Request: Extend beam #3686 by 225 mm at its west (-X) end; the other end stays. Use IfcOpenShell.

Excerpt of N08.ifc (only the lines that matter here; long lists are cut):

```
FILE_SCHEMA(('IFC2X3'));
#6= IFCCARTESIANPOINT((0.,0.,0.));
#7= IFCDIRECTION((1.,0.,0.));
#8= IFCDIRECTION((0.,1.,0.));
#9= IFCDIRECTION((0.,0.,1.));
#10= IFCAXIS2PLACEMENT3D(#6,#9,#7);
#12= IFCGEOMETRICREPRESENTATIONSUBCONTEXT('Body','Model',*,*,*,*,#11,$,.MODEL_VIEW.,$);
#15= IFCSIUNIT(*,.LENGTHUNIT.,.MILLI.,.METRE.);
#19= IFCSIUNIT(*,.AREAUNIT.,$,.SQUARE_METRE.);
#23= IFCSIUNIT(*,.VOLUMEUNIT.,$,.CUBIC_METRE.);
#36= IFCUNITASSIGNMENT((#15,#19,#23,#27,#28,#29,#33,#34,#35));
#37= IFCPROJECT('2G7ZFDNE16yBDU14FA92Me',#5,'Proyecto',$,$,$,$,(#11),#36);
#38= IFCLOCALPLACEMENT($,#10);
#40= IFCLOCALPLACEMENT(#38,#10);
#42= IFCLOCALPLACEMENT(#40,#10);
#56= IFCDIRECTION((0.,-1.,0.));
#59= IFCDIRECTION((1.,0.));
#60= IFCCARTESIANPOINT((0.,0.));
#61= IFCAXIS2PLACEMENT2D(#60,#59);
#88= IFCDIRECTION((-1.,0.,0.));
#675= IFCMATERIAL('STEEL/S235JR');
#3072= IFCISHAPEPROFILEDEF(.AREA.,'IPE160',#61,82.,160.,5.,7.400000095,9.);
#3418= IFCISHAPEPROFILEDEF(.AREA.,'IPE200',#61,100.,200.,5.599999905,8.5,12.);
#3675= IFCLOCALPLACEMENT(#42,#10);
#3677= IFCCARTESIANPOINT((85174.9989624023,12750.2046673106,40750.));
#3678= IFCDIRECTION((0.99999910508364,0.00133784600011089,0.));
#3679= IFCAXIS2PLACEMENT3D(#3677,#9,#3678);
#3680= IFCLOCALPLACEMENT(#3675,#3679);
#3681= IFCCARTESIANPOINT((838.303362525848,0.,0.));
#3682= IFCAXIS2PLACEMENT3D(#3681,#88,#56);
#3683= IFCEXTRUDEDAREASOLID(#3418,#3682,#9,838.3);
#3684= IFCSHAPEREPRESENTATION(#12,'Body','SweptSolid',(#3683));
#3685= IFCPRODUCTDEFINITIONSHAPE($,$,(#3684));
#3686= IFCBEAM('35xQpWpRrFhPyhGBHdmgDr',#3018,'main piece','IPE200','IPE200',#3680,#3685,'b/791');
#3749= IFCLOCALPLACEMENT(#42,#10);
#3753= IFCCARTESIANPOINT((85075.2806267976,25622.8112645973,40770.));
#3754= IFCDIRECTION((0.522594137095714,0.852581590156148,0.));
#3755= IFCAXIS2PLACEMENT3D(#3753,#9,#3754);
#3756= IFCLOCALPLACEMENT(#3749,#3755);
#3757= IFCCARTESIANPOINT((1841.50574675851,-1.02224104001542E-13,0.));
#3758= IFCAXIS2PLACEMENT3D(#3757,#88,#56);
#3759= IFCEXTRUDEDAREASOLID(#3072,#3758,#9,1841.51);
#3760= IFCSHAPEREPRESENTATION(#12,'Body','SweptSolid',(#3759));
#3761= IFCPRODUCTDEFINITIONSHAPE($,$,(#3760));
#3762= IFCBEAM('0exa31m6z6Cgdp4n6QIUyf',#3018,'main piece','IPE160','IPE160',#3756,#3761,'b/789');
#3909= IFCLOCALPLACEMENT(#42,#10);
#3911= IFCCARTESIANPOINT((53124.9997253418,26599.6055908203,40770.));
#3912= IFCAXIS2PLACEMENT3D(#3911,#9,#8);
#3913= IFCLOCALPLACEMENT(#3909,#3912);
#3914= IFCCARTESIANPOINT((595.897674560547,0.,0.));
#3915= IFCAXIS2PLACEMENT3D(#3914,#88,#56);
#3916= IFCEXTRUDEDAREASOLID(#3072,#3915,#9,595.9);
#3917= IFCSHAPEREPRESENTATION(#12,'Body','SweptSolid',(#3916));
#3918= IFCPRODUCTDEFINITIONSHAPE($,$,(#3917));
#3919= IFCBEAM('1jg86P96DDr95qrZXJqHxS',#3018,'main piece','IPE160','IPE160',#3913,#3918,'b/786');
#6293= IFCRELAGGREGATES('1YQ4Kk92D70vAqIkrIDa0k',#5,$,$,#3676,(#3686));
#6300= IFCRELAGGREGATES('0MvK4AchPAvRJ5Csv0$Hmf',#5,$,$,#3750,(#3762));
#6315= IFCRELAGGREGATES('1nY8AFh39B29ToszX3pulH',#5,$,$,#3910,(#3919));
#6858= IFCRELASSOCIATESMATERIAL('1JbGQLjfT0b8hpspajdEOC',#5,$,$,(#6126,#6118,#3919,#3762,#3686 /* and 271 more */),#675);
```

```python
import ifcopenshell
import ifcopenshell.util.representation
import ifcopenshell.util.unit

model = ifcopenshell.open("N08.ifc")
unit_scale = ifcopenshell.util.unit.calculate_unit_scale(model)

member = model.by_guid("35xQpWpRrFhPyhGBHdmgDr")
change = 0.225 / unit_scale

# The extrusion runs towards the end named, so only its depth changes.
body = ifcopenshell.util.representation.get_representation(member, "Model", "Body")
solid = body.Items[0]
old_length = solid.Depth
solid.Depth += change

print(f"length {old_length:g} -> {solid.Depth:g}")

model.write("N08_v2.ifc")
```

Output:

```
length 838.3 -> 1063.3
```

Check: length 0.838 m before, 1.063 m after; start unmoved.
